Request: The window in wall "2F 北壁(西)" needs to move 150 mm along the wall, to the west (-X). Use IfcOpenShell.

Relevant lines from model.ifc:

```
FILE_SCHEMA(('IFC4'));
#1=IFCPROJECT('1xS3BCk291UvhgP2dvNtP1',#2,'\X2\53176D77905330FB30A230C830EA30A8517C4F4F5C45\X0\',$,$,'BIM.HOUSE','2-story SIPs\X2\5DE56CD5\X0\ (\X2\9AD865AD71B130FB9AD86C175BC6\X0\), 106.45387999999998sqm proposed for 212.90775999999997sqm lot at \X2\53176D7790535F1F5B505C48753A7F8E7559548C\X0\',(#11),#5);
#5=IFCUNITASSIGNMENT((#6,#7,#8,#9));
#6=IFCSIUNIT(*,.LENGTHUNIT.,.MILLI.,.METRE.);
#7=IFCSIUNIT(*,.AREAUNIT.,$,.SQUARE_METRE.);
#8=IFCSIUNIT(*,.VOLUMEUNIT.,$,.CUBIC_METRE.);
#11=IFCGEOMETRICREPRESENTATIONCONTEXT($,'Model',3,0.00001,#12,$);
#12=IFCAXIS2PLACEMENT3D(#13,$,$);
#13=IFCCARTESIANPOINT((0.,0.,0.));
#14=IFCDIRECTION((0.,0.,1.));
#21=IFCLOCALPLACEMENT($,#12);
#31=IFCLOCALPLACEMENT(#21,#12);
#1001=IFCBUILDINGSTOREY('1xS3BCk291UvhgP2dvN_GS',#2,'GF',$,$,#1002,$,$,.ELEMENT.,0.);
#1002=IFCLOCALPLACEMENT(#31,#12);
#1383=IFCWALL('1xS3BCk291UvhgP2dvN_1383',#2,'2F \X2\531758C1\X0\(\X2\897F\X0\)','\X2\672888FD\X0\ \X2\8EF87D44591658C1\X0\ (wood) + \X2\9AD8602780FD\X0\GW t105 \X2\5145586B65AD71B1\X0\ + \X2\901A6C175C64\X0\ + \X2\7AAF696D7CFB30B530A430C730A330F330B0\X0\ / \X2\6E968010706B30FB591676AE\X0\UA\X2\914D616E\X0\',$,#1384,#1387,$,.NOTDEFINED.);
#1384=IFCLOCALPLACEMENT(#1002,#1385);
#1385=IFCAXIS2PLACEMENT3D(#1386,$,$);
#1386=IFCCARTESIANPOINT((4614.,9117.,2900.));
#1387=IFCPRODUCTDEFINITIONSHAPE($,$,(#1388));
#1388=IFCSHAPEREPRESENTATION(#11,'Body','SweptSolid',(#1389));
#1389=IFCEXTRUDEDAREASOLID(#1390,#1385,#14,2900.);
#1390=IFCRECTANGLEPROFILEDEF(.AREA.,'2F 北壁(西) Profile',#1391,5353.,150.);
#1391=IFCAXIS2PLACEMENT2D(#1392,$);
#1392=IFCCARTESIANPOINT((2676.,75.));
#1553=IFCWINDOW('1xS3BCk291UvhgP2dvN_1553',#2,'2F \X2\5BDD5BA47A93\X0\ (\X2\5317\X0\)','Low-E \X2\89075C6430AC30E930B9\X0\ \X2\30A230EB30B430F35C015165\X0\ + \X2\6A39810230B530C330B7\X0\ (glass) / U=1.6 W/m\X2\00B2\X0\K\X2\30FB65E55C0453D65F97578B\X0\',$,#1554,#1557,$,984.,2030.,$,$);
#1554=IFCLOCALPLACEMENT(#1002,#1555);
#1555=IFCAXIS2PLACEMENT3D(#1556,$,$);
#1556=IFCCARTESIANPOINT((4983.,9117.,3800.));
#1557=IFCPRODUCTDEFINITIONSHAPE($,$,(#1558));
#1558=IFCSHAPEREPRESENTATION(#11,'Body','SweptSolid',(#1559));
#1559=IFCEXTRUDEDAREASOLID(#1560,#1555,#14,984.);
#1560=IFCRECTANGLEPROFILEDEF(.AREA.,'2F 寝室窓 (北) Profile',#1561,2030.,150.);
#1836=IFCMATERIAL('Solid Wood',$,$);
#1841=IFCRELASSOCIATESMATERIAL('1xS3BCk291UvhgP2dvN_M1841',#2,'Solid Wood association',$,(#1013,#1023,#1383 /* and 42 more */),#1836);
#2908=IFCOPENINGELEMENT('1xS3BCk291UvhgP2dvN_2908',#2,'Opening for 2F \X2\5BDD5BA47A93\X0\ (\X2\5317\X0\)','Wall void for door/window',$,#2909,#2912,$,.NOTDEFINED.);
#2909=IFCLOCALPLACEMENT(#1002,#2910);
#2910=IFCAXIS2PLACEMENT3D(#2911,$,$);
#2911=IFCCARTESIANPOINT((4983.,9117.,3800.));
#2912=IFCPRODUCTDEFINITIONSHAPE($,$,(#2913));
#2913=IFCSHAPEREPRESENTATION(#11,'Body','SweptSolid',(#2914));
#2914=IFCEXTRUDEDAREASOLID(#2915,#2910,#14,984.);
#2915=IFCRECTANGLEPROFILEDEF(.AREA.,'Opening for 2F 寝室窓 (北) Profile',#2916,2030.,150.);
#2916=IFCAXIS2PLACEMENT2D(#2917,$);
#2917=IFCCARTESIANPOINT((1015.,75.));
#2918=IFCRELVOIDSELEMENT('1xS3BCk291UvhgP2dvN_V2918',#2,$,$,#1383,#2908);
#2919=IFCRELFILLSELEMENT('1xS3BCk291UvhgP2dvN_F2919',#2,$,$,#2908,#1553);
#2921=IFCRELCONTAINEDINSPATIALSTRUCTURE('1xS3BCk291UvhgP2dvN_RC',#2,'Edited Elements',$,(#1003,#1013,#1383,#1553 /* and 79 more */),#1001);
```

```python
import ifcopenshell
import ifcopenshell.api.geometry
import ifcopenshell.util.placement
import ifcopenshell.util.unit

model = ifcopenshell.open("model.ifc")
unit_scale = ifcopenshell.util.unit.calculate_unit_scale(model)

window = model.by_guid("1xS3BCk291UvhgP2dvN_1553")
opening = window.FillsVoids[0].RelatingOpeningElement
wall = opening.VoidsElements[0].RelatingBuildingElement

wall_matrix = ifcopenshell.util.placement.get_local_placement(wall.ObjectPlacement)
shift = wall_matrix[:3, 0] * -0.15 / unit_scale
before = ifcopenshell.util.placement.get_local_placement(window.ObjectPlacement)[:3, 3].copy()

# The window is not placed relative to its opening, so move both.
for product in (opening, window):
    matrix = ifcopenshell.util.placement.get_local_placement(product.ObjectPlacement)
    matrix[:3, 3] += shift
    ifcopenshell.api.geometry.edit_object_placement(model, product=product, matrix=matrix, is_si=False)

after = ifcopenshell.util.placement.get_local_placement(window.ObjectPlacement)[:3, 3]
print("window moved by", (after - before).round(3) + 0.0)

model.write("model-out.ifc")
```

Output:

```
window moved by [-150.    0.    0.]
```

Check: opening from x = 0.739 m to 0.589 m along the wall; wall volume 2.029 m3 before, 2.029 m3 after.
